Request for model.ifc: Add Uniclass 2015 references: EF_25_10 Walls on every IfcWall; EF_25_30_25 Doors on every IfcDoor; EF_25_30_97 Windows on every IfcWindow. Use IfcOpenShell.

First a look at what the model holds.

```python
import ifcopenshell

model = ifcopenshell.open("model.ifc")
print(model.schema)
print("classifications:", [c.Name for c in model.by_type("IfcClassification")])
for ifc_class in ("IfcDoor", "IfcRoof", "IfcStair", "IfcWall", "IfcWindow"):
    print(ifc_class, len(model.by_type(ifc_class)))
```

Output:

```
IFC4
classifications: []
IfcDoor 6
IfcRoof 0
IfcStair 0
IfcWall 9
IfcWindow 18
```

```python
import ifcopenshell
import ifcopenshell.api.classification

model = ifcopenshell.open("model.ifc")

system = ifcopenshell.api.classification.add_classification(model, classification="Uniclass 2015")

codes = {
    "IfcWall": ("EF_25_10", "Walls"),
    "IfcDoor": ("EF_25_30_25", "Doors"),
    "IfcWindow": ("EF_25_30_97", "Windows"),
}
for ifc_class, (code, name) in codes.items():
    products = model.by_type(ifc_class)
    ifcopenshell.api.classification.add_reference(
        model, products=products, classification=system, identification=code, name=name
    )
    print(code, len(products))

model.write("model_rev.ifc")
```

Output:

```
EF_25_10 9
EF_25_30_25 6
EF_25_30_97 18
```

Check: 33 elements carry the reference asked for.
